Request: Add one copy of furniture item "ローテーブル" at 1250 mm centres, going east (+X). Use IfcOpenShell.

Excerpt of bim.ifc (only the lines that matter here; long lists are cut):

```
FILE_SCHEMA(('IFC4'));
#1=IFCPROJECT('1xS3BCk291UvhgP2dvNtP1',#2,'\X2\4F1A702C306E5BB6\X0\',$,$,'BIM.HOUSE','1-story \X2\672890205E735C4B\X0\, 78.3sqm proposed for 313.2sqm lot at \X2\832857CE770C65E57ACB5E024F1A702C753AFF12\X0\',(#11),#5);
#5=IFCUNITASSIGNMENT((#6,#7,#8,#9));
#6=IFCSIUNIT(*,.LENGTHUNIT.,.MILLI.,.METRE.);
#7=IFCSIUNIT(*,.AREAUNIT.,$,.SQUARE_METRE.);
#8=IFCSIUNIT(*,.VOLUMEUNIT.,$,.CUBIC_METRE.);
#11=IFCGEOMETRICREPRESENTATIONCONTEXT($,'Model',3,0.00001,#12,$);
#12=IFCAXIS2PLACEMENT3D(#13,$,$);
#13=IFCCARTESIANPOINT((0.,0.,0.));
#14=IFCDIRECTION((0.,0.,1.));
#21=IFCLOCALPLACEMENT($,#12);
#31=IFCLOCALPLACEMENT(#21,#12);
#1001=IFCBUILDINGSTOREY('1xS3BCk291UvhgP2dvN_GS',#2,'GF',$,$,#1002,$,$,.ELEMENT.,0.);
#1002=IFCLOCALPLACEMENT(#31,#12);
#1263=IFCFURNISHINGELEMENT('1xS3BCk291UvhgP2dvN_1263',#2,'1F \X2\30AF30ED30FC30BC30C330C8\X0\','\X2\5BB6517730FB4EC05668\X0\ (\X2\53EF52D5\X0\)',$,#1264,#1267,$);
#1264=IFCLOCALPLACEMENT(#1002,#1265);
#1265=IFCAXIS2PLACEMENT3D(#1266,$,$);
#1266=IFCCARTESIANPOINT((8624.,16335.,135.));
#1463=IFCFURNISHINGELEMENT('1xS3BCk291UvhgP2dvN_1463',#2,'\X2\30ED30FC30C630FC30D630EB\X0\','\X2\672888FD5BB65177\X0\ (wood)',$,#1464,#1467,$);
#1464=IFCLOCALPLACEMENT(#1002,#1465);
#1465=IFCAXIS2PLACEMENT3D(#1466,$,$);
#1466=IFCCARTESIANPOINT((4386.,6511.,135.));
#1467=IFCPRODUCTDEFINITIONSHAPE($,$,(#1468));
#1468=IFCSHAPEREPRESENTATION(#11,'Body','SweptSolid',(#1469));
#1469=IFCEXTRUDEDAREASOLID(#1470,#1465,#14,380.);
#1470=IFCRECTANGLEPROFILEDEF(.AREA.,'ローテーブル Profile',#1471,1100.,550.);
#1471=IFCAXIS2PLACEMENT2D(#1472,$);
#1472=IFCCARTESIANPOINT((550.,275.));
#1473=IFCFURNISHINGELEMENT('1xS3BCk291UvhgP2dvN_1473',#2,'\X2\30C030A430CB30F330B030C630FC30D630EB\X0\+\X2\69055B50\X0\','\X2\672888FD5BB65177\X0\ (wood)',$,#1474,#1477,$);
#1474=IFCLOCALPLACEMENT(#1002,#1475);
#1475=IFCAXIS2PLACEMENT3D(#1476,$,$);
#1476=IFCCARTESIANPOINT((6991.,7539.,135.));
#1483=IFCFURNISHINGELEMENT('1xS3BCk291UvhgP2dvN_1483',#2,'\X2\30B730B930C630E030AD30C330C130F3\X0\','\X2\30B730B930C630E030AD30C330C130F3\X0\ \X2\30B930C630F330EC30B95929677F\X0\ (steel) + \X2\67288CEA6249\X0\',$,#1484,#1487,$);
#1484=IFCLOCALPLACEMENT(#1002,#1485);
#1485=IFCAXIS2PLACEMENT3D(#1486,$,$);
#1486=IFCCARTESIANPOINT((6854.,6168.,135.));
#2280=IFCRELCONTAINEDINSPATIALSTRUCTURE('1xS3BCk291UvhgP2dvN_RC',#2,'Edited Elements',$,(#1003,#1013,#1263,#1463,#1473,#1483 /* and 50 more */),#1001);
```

```python
import numpy as np
import ifcopenshell
import ifcopenshell.api.geometry
import ifcopenshell.api.root
import ifcopenshell.util.element
import ifcopenshell.util.placement
import ifcopenshell.util.unit

model = ifcopenshell.open("bim.ifc")
unit_scale = ifcopenshell.util.unit.calculate_unit_scale(model)


def reuse_history(source, copy):
    """copy_class also copies each property set's owner history, people and application; keep the originals."""
    for rel in copy.IsDefinedBy:
        if rel.is_a("IfcRelDefinesByProperties") and (history := rel.RelatingPropertyDefinition.OwnerHistory):
            rel.RelatingPropertyDefinition.OwnerHistory = source.OwnerHistory
            ifcopenshell.util.element.remove_deep2(model, history)


source = model.by_id(1463)
base = ifcopenshell.util.placement.get_local_placement(source.ObjectPlacement)
step = np.array([1.0, 0.0, 0.0]) * 1.25 / unit_scale

for i in range(1, 2):
    copy = ifcopenshell.api.root.copy_class(model, product=source)
    copy.Representation = ifcopenshell.util.element.copy_deep(
        model, source.Representation, exclude=["IfcGeometricRepresentationContext", "IfcRepresentationMap"]
    )
    reuse_history(source, copy)
    matrix = base.copy()
    matrix[:3, 3] += i * step
    print("added at", matrix[:3, 3].round(3) + 0.0)
    ifcopenshell.api.geometry.edit_object_placement(model, product=copy, matrix=matrix, is_si=False)

model.write("bim-out.ifc")
```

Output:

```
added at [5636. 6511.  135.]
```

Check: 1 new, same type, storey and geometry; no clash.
